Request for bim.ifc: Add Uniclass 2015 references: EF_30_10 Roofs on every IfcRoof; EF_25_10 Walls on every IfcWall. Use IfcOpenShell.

First a look at what the model holds.

```python
import ifcopenshell

model = ifcopenshell.open("bim.ifc")
print(model.schema)
print("classifications:", [c.Name for c in model.by_type("IfcClassification")])
for ifc_class in ("IfcDoor", "IfcRoof", "IfcStair", "IfcWall", "IfcWindow"):
    print(ifc_class, len(model.by_type(ifc_class)))
```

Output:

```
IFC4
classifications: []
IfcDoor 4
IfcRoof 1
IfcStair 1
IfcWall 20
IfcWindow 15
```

```python
import ifcopenshell
import ifcopenshell.api.classification

model = ifcopenshell.open("bim.ifc")

system = ifcopenshell.api.classification.add_classification(model, classification="Uniclass 2015")

codes = {
    "IfcRoof": ("EF_30_10", "Roofs"),
    "IfcWall": ("EF_25_10", "Walls"),
}
for ifc_class, (code, name) in codes.items():
    products = model.by_type(ifc_class)
    ifcopenshell.api.classification.add_reference(
        model, products=products, classification=system, identification=code, name=name
    )
    print(code, len(products))

model.write("bim_edited.ifc")
```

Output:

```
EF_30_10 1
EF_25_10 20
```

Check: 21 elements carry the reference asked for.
